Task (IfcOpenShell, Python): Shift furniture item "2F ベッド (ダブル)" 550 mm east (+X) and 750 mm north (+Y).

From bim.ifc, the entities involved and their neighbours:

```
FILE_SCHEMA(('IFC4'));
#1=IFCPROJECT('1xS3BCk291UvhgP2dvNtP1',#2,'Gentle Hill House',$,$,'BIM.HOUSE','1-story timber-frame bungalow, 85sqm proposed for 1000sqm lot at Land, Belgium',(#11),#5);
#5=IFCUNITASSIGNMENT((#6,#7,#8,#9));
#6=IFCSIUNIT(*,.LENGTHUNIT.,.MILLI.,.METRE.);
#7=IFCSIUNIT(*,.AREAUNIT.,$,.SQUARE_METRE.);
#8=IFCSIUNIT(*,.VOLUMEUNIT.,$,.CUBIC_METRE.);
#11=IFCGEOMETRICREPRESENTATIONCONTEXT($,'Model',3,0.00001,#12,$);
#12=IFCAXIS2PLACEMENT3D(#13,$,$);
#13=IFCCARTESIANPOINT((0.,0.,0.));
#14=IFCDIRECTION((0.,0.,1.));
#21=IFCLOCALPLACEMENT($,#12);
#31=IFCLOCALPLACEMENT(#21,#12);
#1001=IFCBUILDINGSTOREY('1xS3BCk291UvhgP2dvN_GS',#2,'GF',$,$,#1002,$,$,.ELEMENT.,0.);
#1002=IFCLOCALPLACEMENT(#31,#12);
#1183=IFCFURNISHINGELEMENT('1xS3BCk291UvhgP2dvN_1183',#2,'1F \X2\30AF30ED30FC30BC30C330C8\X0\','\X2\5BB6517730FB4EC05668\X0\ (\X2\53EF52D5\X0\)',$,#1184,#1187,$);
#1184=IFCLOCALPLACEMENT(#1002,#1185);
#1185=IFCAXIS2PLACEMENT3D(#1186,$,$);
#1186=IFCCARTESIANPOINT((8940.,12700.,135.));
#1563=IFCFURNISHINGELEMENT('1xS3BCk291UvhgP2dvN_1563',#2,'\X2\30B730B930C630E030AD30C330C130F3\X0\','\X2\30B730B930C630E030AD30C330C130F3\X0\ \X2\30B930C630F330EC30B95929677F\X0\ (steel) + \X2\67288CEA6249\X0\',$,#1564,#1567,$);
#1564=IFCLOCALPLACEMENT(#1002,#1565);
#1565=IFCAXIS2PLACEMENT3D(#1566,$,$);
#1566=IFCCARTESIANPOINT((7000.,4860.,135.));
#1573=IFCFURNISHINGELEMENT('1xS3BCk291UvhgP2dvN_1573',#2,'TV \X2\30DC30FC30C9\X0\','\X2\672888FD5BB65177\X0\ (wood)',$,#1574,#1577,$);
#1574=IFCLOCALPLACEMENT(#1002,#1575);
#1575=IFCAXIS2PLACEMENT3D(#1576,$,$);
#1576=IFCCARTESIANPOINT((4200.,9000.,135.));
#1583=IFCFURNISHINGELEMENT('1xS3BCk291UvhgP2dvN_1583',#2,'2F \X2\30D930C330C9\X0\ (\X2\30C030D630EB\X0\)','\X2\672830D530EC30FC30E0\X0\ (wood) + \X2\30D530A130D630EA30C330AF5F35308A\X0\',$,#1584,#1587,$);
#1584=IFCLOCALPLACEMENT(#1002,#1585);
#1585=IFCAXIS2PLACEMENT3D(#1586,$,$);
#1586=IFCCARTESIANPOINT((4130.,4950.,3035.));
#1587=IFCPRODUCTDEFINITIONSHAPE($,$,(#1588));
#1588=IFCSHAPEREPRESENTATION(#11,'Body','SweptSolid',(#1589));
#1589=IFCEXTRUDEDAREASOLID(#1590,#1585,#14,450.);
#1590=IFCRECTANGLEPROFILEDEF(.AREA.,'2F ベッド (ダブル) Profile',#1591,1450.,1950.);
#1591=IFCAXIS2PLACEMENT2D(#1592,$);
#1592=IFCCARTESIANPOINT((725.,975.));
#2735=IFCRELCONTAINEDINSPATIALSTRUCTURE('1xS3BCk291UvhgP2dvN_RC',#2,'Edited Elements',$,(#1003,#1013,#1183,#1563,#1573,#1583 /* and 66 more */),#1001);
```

```python
import ifcopenshell
import ifcopenshell.api.geometry
import ifcopenshell.util.placement

model = ifcopenshell.open("bim.ifc")

item = model.by_guid("1xS3BCk291UvhgP2dvN_1583")
matrix = ifcopenshell.util.placement.get_local_placement(item.ObjectPlacement)
matrix[0, 3] += 550.0
matrix[1, 3] += 750.0
ifcopenshell.api.geometry.edit_object_placement(model, product=item, matrix=matrix, is_si=False)

print(ifcopenshell.util.placement.get_local_placement(item.ObjectPlacement).round(3) + 0.0)

model.write("bim_edited.ifc")
```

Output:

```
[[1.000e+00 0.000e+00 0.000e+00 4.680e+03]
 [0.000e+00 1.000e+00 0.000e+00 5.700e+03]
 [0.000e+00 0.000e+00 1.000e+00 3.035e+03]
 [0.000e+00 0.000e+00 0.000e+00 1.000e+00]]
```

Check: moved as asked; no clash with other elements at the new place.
